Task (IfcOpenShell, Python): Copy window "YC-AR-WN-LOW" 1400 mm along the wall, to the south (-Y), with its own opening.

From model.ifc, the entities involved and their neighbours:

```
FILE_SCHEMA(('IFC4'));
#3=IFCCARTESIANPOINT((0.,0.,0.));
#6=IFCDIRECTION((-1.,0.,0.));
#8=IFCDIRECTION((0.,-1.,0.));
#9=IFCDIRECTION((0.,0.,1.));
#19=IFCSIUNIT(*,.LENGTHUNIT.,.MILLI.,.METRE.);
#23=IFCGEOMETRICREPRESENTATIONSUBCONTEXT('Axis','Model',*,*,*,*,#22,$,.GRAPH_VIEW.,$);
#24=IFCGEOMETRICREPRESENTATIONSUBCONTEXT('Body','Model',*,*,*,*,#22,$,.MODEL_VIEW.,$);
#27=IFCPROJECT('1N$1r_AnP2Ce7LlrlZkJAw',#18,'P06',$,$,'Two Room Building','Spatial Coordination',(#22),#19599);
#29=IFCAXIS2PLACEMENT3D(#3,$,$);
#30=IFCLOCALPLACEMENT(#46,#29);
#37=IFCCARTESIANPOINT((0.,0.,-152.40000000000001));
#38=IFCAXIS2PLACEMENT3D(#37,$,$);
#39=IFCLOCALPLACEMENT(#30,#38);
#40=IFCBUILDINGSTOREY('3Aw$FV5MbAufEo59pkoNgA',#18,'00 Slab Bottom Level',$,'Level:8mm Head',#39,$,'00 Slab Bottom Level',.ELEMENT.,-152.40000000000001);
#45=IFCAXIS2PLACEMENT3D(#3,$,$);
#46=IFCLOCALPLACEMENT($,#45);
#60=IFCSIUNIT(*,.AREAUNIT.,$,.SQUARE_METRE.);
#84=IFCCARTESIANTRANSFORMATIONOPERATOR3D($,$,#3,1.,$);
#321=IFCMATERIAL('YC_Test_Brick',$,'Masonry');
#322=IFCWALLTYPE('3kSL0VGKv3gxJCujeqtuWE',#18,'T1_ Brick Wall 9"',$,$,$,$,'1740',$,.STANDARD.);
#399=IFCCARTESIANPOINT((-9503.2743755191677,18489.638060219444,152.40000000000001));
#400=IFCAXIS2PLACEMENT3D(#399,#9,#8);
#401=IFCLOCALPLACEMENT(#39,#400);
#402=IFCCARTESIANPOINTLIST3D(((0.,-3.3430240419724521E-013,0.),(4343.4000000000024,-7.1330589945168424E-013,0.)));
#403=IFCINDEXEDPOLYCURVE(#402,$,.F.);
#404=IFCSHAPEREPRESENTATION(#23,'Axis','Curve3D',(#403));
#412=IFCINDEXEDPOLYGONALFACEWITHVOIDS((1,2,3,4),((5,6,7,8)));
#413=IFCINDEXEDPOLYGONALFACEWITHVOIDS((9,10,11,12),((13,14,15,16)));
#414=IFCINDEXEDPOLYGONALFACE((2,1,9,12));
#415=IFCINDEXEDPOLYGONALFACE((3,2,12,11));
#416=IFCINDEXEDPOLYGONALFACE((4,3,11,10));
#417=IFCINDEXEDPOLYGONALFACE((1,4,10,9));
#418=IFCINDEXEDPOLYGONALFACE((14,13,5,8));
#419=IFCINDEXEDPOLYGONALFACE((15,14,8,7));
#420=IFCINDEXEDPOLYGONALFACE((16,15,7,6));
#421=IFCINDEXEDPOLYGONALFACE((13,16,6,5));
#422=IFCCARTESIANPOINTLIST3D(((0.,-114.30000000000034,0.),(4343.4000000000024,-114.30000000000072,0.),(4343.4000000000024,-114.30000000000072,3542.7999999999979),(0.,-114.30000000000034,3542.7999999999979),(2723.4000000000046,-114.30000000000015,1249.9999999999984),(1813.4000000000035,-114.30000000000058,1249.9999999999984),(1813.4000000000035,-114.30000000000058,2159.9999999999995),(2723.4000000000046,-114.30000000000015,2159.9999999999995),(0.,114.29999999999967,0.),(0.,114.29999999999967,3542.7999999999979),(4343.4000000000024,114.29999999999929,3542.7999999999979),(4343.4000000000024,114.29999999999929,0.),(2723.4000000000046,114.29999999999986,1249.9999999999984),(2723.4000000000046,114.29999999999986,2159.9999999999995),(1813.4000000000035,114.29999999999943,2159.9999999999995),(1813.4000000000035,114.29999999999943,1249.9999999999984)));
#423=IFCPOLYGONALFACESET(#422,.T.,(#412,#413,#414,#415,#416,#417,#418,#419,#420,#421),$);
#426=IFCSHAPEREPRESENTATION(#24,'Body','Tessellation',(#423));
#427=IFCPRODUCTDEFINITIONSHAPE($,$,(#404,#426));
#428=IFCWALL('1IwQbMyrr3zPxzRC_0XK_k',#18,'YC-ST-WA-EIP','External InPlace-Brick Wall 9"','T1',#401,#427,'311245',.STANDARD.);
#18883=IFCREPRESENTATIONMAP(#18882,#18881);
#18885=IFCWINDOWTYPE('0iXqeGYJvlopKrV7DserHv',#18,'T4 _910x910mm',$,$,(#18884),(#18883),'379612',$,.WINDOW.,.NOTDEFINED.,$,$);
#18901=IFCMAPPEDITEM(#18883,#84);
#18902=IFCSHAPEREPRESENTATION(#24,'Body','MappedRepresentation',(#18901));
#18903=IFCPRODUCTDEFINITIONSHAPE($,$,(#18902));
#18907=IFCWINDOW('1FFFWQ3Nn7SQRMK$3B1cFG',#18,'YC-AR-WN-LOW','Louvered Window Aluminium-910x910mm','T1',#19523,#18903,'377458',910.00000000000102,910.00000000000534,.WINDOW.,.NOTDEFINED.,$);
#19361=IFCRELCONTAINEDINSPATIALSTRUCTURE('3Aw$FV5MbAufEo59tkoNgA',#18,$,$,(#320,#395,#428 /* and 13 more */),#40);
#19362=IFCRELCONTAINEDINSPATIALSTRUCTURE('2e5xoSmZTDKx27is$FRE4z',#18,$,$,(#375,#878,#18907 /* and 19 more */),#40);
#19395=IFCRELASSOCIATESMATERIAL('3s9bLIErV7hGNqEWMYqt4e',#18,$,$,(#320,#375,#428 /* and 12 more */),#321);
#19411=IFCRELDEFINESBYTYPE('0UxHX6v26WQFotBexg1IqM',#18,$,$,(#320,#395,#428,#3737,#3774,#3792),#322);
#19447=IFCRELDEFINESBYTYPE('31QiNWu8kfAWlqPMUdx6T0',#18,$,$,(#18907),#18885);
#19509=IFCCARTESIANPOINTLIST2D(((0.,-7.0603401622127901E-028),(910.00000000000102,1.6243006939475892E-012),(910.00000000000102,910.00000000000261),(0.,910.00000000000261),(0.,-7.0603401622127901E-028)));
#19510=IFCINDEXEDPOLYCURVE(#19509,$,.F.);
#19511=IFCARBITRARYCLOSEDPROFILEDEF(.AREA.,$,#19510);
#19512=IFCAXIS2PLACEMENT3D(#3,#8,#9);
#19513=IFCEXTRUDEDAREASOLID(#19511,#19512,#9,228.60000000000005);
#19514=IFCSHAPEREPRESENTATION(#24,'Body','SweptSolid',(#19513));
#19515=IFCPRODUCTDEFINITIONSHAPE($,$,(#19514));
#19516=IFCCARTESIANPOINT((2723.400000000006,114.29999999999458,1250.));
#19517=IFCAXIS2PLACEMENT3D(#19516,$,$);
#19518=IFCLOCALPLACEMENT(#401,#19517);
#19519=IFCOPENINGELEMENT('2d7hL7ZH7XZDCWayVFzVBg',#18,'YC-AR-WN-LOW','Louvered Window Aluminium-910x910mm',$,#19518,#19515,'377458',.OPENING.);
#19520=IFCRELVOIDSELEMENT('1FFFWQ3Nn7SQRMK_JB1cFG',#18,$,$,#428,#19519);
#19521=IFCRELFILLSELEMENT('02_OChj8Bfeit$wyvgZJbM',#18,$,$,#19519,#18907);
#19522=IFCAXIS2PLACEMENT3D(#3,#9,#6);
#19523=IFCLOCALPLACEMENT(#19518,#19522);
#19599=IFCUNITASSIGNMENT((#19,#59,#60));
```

```python
import ifcopenshell
import ifcopenshell.api.feature
import ifcopenshell.api.geometry
import ifcopenshell.api.root
import ifcopenshell.geom
import ifcopenshell.util.element
import ifcopenshell.util.placement
import ifcopenshell.util.shape
import ifcopenshell.util.unit

model = ifcopenshell.open("model.ifc")
unit_scale = ifcopenshell.util.unit.calculate_unit_scale(model)
settings = ifcopenshell.geom.settings()


def volume(element):
    """Net volume in cubic metres, openings subtracted."""
    shape = ifcopenshell.geom.create_shape(settings, element)
    return ifcopenshell.util.shape.get_volume(shape.geometry)


def reuse_history(source, copy):
    """copy_class also copies each property set's owner history, people and application; keep the originals."""
    for rel in copy.IsDefinedBy:
        if rel.is_a("IfcRelDefinesByProperties") and (history := rel.RelatingPropertyDefinition.OwnerHistory):
            rel.RelatingPropertyDefinition.OwnerHistory = source.OwnerHistory
            ifcopenshell.util.element.remove_deep2(model, history)


window = model.by_id(18907)
opening = window.FillsVoids[0].RelatingOpeningElement
wall = opening.VoidsElements[0].RelatingBuildingElement
before = volume(wall)
shift = ifcopenshell.util.placement.get_local_placement(wall.ObjectPlacement)[:3, 0] * 1.4 / unit_scale

# copy_class copies the void relationship, type, container and properties, but no geometry.
new_opening = ifcopenshell.api.root.copy_class(model, product=opening)
new_opening.Representation = ifcopenshell.util.element.copy_deep(
    model, opening.Representation, exclude=["IfcGeometricRepresentationContext", "IfcRepresentationMap"]
)
new_opening.Tag = None
new_window = ifcopenshell.api.root.copy_class(model, product=window)
new_window.Representation = ifcopenshell.util.element.copy_deep(
    model, window.Representation, exclude=["IfcGeometricRepresentationContext", "IfcRepresentationMap"]
)
new_window.Tag = None
reuse_history(window, new_window)
ifcopenshell.api.feature.add_filling(model, opening=new_opening, element=new_window)

for old, new in ((opening, new_opening), (window, new_window)):
    matrix = ifcopenshell.util.placement.get_local_placement(old.ObjectPlacement)
    matrix[:3, 3] += shift
    ifcopenshell.api.geometry.edit_object_placement(model, product=new, matrix=matrix, is_si=False)

after = volume(wall)

print(f"wall volume {before:.3f} -> {after:.3f} m3")

model.write("model_v2.ifc")
```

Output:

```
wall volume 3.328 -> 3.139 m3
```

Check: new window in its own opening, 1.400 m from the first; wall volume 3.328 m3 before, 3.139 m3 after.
